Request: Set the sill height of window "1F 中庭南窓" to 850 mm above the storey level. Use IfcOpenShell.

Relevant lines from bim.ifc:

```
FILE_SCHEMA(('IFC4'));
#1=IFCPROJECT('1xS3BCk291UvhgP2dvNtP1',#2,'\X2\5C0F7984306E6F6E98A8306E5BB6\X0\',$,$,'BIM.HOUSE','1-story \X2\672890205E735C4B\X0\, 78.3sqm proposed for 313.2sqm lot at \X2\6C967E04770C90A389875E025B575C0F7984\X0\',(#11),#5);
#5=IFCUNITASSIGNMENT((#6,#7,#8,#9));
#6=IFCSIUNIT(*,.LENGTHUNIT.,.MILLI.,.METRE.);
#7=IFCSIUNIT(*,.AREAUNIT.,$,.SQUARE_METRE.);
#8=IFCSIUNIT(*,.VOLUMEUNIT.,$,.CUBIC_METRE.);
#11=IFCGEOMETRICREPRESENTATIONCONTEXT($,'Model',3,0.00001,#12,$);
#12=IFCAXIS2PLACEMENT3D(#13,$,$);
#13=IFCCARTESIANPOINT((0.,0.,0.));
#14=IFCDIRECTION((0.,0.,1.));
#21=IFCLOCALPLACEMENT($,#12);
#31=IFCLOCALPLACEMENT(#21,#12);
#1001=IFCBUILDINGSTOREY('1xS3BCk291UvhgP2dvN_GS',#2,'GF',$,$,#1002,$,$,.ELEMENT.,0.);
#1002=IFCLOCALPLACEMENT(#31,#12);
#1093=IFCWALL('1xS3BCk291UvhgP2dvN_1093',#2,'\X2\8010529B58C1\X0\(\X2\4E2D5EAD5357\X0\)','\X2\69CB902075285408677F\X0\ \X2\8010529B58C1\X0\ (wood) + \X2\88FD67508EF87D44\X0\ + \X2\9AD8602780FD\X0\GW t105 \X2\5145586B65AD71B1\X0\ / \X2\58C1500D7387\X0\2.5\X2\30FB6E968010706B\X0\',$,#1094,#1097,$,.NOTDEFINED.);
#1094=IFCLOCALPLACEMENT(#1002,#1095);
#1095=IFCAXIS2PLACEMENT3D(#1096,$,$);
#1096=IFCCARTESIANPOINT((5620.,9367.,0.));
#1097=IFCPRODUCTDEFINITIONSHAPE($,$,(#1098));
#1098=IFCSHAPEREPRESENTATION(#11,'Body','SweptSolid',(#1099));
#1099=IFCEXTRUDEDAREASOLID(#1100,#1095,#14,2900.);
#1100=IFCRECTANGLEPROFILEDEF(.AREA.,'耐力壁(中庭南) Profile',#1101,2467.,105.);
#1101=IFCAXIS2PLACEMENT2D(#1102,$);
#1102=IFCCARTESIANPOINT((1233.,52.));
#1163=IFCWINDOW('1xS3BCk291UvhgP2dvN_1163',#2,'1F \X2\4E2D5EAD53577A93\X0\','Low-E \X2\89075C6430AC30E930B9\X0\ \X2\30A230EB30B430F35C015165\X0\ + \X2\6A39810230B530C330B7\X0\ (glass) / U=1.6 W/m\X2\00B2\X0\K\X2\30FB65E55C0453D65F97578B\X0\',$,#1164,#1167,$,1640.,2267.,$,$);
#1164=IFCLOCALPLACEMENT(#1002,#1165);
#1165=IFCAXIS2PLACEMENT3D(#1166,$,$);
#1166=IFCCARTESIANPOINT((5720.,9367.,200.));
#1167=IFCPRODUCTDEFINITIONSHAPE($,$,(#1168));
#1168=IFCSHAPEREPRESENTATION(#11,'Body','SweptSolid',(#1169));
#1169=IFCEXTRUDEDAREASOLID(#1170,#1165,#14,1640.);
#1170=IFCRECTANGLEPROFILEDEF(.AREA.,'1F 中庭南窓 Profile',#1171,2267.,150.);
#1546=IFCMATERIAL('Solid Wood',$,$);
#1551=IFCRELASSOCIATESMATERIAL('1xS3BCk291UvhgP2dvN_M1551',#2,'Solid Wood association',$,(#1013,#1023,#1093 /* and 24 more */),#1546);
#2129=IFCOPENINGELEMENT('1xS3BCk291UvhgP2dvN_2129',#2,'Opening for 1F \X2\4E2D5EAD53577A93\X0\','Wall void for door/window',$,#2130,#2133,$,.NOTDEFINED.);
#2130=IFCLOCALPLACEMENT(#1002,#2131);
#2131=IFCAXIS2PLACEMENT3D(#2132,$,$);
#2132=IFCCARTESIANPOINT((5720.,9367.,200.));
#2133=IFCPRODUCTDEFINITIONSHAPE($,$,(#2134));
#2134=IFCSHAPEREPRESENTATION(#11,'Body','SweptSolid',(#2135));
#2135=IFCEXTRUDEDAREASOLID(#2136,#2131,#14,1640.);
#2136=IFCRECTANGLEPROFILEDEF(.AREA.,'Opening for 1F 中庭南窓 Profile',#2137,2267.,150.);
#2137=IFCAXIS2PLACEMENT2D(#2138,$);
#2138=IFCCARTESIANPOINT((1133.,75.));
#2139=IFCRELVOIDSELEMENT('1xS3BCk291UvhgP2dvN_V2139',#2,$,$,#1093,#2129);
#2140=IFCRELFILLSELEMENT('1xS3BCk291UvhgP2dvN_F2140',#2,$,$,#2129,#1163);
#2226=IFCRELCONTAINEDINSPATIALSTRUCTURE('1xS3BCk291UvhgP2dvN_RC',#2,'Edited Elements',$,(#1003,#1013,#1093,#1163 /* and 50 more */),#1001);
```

```python
import numpy as np
import ifcopenshell
import ifcopenshell.api.geometry
import ifcopenshell.geom
import ifcopenshell.util.element
import ifcopenshell.util.placement
import ifcopenshell.util.shape
import ifcopenshell.util.unit

model = ifcopenshell.open("bim.ifc")
unit_scale = ifcopenshell.util.unit.calculate_unit_scale(model)

window = model.by_id(1163)
opening = window.FillsVoids[0].RelatingOpeningElement
storey = ifcopenshell.util.element.get_container(window, ifc_class="IfcBuildingStorey")
level = ifcopenshell.util.placement.get_local_placement(storey.ObjectPlacement)[2, 3]

# The opening's origin need not be at the sill, so measure its lowest point.
shape = ifcopenshell.geom.create_shape(ifcopenshell.geom.settings(), opening)
bottom = ifcopenshell.util.shape.get_shape_bottom_elevation(shape, shape.geometry) / unit_scale
dz = level + 0.85 / unit_scale - bottom

shift = np.array([0.0, 0.0, dz])
# The window is not placed relative to its opening, so move both.
for product in (opening, window):
    matrix = ifcopenshell.util.placement.get_local_placement(product.ObjectPlacement)
    matrix[:3, 3] += shift
    ifcopenshell.api.geometry.edit_object_placement(model, product=product, matrix=matrix, is_si=False)

print(f"moved by {dz * unit_scale:+.3f} m")

model.write("bim_rev.ifc")
```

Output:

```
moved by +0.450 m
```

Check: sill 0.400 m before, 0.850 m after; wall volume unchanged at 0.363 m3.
